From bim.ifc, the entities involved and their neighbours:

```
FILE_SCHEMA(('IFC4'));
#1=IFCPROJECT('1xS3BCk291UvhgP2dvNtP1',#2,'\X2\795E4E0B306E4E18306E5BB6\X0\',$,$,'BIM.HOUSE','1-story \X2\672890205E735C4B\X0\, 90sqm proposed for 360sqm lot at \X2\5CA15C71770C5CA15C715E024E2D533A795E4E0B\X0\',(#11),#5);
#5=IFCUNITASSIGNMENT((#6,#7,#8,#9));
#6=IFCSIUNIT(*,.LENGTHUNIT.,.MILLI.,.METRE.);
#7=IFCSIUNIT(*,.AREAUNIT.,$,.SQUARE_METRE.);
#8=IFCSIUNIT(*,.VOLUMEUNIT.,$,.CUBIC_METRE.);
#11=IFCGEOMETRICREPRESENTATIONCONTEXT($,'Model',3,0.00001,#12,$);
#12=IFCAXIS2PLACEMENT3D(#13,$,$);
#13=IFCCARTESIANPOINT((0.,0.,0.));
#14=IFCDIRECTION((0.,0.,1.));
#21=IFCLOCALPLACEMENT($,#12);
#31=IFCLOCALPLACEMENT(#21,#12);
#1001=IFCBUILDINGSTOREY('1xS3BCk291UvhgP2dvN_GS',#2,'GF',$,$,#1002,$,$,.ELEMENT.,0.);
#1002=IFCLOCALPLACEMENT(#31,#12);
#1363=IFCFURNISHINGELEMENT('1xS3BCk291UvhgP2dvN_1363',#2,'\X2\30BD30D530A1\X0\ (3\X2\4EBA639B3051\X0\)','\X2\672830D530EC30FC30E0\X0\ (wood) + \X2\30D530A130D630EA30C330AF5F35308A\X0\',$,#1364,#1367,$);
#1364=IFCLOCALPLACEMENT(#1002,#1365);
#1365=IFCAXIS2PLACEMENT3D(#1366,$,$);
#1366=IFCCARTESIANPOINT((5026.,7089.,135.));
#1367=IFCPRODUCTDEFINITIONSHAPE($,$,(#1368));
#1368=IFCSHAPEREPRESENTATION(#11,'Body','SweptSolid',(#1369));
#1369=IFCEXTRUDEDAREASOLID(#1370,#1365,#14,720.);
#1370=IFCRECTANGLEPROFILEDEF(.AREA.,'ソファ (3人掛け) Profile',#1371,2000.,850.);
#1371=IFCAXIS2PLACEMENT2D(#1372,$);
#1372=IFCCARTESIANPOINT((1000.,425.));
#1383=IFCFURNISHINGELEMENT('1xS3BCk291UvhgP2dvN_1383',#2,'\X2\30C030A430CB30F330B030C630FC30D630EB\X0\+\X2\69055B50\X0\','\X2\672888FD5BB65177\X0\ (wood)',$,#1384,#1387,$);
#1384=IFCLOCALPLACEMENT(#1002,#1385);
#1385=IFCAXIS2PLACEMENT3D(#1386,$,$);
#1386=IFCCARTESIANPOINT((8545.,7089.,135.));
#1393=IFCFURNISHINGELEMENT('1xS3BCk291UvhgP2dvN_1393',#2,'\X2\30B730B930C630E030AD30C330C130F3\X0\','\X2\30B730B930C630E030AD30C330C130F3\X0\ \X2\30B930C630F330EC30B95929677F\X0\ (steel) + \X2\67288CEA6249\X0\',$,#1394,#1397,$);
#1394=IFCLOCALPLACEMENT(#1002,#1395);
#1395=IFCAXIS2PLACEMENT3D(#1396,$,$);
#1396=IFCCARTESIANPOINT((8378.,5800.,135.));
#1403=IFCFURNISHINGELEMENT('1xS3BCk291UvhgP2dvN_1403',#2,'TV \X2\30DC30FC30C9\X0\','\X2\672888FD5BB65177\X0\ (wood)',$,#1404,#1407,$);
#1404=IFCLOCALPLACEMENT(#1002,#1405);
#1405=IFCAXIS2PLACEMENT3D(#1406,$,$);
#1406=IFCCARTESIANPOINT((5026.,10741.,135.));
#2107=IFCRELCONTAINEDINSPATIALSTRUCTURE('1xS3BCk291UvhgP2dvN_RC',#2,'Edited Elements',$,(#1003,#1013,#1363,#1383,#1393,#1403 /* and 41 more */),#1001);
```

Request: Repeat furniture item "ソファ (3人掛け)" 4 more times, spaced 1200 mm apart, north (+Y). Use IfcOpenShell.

```python
import numpy as np
import ifcopenshell
import ifcopenshell.api.geometry
import ifcopenshell.api.root
import ifcopenshell.util.element
import ifcopenshell.util.placement
import ifcopenshell.util.unit

model = ifcopenshell.open("bim.ifc")
unit_scale = ifcopenshell.util.unit.calculate_unit_scale(model)


def reuse_history(source, copy):
    """copy_class also copies each property set's owner history, people and application; keep the originals."""
    for rel in copy.IsDefinedBy:
        if rel.is_a("IfcRelDefinesByProperties") and (history := rel.RelatingPropertyDefinition.OwnerHistory):
            rel.RelatingPropertyDefinition.OwnerHistory = source.OwnerHistory
            ifcopenshell.util.element.remove_deep2(model, history)


source = model.by_guid("1xS3BCk291UvhgP2dvN_1363")
base = ifcopenshell.util.placement.get_local_placement(source.ObjectPlacement)
step = np.array([0.0, 1.0, 0.0]) * 1.2 / unit_scale

for i in range(1, 5):
    copy = ifcopenshell.api.root.copy_class(model, product=source)
    copy.Representation = ifcopenshell.util.element.copy_deep(
        model, source.Representation, exclude=["IfcGeometricRepresentationContext", "IfcRepresentationMap"]
    )
    reuse_history(source, copy)
    matrix = base.copy()
    matrix[:3, 3] += i * step
    print("added at", matrix[:3, 3].round(3) + 0.0)
    ifcopenshell.api.geometry.edit_object_placement(model, product=copy, matrix=matrix, is_si=False)

model.write("bim_v2.ifc")
```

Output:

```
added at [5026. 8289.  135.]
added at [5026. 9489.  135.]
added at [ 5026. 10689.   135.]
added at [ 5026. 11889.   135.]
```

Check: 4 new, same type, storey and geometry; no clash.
